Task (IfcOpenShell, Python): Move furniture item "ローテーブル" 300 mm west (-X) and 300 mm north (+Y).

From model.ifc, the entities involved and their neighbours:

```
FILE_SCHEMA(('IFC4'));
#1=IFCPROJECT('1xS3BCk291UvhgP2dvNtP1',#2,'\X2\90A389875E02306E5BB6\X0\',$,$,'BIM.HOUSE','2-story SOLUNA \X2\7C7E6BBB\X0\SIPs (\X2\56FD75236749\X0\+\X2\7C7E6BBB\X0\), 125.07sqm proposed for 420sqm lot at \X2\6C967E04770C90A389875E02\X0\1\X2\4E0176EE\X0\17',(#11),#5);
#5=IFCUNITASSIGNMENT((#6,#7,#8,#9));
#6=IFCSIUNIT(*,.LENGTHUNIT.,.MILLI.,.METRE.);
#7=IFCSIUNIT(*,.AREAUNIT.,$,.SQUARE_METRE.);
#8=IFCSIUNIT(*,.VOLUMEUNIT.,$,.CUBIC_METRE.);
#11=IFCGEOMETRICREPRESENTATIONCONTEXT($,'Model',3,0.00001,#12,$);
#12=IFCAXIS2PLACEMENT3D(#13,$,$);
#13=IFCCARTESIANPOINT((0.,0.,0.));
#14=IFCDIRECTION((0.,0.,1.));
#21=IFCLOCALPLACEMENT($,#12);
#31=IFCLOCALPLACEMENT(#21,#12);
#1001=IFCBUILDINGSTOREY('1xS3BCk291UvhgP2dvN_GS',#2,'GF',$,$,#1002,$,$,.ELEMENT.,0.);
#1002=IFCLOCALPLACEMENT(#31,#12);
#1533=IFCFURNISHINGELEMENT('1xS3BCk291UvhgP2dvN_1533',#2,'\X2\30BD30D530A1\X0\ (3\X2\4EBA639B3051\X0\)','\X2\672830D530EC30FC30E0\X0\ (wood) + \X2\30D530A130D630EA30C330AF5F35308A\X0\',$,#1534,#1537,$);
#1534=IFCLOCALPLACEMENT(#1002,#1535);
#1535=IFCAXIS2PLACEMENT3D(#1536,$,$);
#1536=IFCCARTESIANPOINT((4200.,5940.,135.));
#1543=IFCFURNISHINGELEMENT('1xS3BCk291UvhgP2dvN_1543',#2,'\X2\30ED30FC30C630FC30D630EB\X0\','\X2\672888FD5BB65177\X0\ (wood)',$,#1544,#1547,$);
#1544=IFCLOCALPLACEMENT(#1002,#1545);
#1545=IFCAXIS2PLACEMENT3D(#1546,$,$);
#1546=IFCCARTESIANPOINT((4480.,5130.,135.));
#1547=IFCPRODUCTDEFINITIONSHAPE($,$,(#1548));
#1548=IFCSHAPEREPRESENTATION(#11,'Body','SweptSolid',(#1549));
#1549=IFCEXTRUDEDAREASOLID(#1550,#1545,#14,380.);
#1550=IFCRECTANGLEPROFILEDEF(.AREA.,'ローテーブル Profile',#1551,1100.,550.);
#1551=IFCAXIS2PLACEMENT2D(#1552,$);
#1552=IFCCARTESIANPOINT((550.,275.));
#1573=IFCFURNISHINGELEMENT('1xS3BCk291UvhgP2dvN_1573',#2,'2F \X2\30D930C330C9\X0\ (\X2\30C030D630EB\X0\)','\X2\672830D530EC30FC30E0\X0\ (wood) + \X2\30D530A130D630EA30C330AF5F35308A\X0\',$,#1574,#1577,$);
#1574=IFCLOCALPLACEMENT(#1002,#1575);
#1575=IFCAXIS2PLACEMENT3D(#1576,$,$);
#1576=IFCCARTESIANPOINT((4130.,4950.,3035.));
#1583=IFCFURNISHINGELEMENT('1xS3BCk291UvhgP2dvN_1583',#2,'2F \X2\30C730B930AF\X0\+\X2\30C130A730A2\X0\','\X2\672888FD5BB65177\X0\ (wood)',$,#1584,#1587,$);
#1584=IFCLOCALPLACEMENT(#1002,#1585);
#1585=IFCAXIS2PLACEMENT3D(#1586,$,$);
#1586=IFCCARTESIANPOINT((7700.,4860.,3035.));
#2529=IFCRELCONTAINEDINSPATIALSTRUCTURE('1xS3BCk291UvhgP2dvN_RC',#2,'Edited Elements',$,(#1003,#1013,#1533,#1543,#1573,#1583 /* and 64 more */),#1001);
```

```python
import ifcopenshell
import ifcopenshell.api.geometry
import ifcopenshell.util.placement
import ifcopenshell.util.unit

model = ifcopenshell.open("model.ifc")
unit_scale = ifcopenshell.util.unit.calculate_unit_scale(model)

item = model.by_id(1543)
matrix = ifcopenshell.util.placement.get_local_placement(item.ObjectPlacement)
matrix[0, 3] -= 0.3 / unit_scale
matrix[1, 3] += 0.3 / unit_scale
ifcopenshell.api.geometry.edit_object_placement(model, product=item, matrix=matrix, is_si=False)

print(ifcopenshell.util.placement.get_local_placement(item.ObjectPlacement).round(3) + 0.0)

model.write("model_updated.ifc")
```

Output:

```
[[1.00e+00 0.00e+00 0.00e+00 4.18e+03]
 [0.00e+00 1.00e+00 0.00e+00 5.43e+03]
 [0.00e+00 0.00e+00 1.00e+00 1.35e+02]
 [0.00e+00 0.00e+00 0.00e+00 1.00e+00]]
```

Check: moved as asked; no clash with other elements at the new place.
